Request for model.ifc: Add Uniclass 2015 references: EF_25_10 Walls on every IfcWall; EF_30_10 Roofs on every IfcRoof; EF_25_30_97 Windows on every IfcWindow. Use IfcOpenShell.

First a look at what the model holds.

```python
import ifcopenshell

model = ifcopenshell.open("model.ifc")
print(model.schema)
print("classifications:", [c.Name for c in model.by_type("IfcClassification")])
for ifc_class in ("IfcDoor", "IfcRoof", "IfcStair", "IfcWall", "IfcWindow"):
    print(ifc_class, len(model.by_type(ifc_class)))
```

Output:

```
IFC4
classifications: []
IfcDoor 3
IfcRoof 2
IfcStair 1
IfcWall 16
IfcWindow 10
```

```python
import ifcopenshell
import ifcopenshell.api.classification

model = ifcopenshell.open("model.ifc")

system = ifcopenshell.api.classification.add_classification(model, classification="Uniclass 2015")

codes = {
    "IfcWall": ("EF_25_10", "Walls"),
    "IfcRoof": ("EF_30_10", "Roofs"),
    "IfcWindow": ("EF_25_30_97", "Windows"),
}
for ifc_class, (code, name) in codes.items():
    products = model.by_type(ifc_class)
    ifcopenshell.api.classification.add_reference(
        model, products=products, classification=system, identification=code, name=name
    )
    print(code, len(products))

model.write("model-out.ifc")
```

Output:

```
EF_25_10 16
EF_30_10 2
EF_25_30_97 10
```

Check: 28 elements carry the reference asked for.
